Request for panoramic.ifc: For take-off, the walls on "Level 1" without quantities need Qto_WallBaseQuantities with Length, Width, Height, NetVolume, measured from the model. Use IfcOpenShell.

First a look at what the model holds.

```python
import ifcopenshell
import ifcopenshell.util.element
import ifcopenshell.util.unit

model = ifcopenshell.open("panoramic.ifc")
print(model.schema)
for unit_type in ("LENGTHUNIT", "AREAUNIT", "VOLUMEUNIT"):
    print(unit_type, ifcopenshell.util.unit.calculate_unit_scale(model, unit_type))
storey = next(s for s in model.by_type("IfcBuildingStorey") if s.Name == "Level 1")
walls = [e for e in ifcopenshell.util.element.get_decomposition(storey) if e.is_a("IfcWall")]
for e in sorted(walls, key=lambda e: e.id()):
    print(e.id(), e.is_a(), e.Name, list(ifcopenshell.util.element.get_psets(e, qtos_only=True)), sep=" | ")
```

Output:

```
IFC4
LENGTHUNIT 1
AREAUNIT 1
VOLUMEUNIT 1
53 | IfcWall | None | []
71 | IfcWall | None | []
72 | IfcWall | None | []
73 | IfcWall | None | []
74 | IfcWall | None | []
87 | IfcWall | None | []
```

```python
import ifcopenshell
import ifcopenshell.api.pset
import ifcopenshell.geom
import ifcopenshell.util.element
import ifcopenshell.util.shape
import ifcopenshell.util.unit

model = ifcopenshell.open("panoramic.ifc")
unit_scale = ifcopenshell.util.unit.calculate_unit_scale(model)
volume_scale = ifcopenshell.util.unit.calculate_unit_scale(model, "VOLUMEUNIT")
settings = ifcopenshell.geom.settings()

storey = next(s for s in model.by_type("IfcBuildingStorey") if s.Name == "Level 1")
walls = [e for e in ifcopenshell.util.element.get_decomposition(storey) if e.is_a("IfcWall")]

for e in sorted(walls, key=lambda e: e.id()):
    if ifcopenshell.util.element.get_psets(e, qtos_only=True, should_inherit=False):
        continue
    # Geometry comes back in metres, in the element's own axes.
    shape = ifcopenshell.geom.create_shape(settings, e)
    values = {
        "Length": ifcopenshell.util.shape.get_x(shape.geometry) / unit_scale,
        "Width": ifcopenshell.util.shape.get_y(shape.geometry) / unit_scale,
        "Height": ifcopenshell.util.shape.get_z(shape.geometry) / unit_scale,
        "NetVolume": ifcopenshell.util.shape.get_volume(shape.geometry) / volume_scale,
    }
    qto = ifcopenshell.api.pset.add_qto(model, product=e, name="Qto_WallBaseQuantities")
    ifcopenshell.api.pset.edit_qto(model, qto=qto, properties=values)
    print(e.id(), {k: round(v, 3) for k, v in values.items()})

model.write("panoramic_v2.ifc")
```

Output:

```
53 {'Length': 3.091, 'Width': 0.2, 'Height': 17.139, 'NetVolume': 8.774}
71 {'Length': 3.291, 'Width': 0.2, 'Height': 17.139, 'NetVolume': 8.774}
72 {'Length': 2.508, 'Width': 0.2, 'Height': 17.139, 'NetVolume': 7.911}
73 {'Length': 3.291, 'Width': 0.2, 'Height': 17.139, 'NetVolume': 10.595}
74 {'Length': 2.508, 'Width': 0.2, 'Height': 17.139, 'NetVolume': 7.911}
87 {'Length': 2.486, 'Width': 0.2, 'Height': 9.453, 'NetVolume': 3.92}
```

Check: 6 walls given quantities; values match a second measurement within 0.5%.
